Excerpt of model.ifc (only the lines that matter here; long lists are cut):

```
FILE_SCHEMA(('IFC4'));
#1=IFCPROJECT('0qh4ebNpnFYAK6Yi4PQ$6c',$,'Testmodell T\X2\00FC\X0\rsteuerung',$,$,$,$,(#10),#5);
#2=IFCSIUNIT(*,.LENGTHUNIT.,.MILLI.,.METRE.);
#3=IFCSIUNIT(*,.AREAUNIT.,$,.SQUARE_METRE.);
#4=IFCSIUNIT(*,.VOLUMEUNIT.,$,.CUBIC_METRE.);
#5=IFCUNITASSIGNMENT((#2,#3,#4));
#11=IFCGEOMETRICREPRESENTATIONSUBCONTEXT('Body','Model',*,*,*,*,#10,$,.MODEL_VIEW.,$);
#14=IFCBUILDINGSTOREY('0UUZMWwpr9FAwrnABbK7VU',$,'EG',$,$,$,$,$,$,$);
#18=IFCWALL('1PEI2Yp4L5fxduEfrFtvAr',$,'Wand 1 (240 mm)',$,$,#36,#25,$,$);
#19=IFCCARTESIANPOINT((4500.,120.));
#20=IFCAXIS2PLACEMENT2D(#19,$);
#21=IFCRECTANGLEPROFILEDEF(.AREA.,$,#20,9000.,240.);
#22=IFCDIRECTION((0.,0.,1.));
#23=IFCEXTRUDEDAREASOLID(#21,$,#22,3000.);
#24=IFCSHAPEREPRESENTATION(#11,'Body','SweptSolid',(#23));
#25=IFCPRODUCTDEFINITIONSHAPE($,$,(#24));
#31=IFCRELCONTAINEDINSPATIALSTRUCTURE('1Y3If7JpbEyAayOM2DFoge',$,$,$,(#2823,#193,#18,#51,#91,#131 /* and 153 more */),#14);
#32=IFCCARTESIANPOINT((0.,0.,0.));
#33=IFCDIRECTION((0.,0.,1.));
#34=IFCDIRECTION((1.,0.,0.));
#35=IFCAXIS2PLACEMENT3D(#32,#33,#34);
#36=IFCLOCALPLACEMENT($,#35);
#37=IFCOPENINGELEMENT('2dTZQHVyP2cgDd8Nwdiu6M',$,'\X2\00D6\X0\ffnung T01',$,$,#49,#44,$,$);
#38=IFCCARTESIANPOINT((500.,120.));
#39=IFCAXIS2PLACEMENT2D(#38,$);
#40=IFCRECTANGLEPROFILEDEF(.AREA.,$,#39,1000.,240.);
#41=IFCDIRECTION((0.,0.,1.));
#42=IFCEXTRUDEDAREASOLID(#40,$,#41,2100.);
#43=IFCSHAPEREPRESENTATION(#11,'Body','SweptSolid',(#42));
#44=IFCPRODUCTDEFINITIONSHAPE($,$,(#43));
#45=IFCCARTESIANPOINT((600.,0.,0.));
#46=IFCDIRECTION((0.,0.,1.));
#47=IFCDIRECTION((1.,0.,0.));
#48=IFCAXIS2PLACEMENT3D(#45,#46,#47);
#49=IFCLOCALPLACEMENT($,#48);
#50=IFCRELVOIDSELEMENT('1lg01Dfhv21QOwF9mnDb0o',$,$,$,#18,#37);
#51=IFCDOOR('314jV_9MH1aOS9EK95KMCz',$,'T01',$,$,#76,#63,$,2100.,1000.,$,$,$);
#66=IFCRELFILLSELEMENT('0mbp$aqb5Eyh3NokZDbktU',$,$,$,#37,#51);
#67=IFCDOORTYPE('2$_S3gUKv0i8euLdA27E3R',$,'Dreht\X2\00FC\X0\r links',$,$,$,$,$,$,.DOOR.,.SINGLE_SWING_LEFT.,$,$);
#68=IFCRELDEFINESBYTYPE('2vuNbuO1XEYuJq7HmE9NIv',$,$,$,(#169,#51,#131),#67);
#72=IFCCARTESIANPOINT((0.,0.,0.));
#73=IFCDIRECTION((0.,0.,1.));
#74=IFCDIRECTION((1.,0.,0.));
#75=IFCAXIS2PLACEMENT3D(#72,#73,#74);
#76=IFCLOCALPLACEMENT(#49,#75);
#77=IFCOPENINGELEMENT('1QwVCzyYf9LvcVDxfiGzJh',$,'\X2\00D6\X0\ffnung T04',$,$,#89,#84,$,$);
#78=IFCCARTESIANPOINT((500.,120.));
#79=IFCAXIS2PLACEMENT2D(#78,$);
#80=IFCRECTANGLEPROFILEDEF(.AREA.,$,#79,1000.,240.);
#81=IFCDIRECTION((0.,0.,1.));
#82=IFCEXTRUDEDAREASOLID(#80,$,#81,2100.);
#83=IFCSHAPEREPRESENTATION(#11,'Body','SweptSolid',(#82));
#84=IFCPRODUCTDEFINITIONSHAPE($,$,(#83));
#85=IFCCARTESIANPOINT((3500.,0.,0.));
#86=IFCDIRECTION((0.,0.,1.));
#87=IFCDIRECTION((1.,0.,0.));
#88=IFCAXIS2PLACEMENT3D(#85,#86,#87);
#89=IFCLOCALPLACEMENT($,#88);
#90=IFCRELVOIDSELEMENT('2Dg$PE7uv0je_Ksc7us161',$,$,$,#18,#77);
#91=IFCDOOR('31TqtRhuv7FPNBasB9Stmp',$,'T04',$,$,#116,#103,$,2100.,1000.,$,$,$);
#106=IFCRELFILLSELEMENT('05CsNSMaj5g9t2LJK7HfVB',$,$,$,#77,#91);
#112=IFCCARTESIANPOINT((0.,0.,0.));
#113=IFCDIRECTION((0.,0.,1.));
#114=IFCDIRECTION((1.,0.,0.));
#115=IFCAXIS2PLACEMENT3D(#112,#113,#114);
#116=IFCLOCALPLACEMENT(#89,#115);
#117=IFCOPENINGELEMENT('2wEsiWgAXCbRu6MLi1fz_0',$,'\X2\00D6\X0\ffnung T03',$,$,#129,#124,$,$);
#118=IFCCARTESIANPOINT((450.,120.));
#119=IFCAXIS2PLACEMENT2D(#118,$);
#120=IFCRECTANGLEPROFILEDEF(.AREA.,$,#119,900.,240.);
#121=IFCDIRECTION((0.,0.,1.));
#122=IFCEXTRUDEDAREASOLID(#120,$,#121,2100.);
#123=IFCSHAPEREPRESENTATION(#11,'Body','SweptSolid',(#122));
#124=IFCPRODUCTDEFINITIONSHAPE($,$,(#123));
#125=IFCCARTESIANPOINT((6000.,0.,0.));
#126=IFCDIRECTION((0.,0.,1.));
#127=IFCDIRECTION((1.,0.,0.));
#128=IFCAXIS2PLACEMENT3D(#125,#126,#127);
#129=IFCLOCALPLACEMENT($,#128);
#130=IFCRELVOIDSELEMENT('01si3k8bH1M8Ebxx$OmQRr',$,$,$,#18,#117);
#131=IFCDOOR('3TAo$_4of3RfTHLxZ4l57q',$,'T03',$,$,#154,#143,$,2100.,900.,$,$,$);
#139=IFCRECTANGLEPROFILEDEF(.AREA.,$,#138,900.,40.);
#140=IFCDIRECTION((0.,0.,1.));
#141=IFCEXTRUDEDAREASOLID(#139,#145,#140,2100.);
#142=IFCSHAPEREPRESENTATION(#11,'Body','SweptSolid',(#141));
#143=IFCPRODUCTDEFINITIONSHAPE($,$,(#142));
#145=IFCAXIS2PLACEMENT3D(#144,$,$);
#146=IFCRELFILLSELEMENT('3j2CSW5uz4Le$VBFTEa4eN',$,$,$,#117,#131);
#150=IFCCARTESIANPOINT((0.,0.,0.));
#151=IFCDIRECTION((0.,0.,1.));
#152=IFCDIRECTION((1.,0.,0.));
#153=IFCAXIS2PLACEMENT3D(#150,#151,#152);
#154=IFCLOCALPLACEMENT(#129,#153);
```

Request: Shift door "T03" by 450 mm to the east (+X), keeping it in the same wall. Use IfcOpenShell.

```python
import ifcopenshell
import ifcopenshell.api.geometry
import ifcopenshell.util.placement

model = ifcopenshell.open("model.ifc")

door = model.by_guid("3TAo$_4of3RfTHLxZ4l57q")
opening = door.FillsVoids[0].RelatingOpeningElement
wall = opening.VoidsElements[0].RelatingBuildingElement

wall_matrix = ifcopenshell.util.placement.get_local_placement(wall.ObjectPlacement)
shift = wall_matrix[:3, 0] * 450.0
before = ifcopenshell.util.placement.get_local_placement(door.ObjectPlacement)[:3, 3].copy()

# The door is placed relative to its opening, so it follows when the opening moves.
matrix = ifcopenshell.util.placement.get_local_placement(opening.ObjectPlacement)
matrix[:3, 3] += shift
ifcopenshell.api.geometry.edit_object_placement(
    model, product=opening, matrix=matrix, is_si=False, should_transform_children=True
)

after = ifcopenshell.util.placement.get_local_placement(door.ObjectPlacement)[:3, 3]
print("door moved by", (after - before).round(3) + 0.0)

model.write("model_edited.ifc")
```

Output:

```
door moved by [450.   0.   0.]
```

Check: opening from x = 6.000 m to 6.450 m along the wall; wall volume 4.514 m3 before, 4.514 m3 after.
